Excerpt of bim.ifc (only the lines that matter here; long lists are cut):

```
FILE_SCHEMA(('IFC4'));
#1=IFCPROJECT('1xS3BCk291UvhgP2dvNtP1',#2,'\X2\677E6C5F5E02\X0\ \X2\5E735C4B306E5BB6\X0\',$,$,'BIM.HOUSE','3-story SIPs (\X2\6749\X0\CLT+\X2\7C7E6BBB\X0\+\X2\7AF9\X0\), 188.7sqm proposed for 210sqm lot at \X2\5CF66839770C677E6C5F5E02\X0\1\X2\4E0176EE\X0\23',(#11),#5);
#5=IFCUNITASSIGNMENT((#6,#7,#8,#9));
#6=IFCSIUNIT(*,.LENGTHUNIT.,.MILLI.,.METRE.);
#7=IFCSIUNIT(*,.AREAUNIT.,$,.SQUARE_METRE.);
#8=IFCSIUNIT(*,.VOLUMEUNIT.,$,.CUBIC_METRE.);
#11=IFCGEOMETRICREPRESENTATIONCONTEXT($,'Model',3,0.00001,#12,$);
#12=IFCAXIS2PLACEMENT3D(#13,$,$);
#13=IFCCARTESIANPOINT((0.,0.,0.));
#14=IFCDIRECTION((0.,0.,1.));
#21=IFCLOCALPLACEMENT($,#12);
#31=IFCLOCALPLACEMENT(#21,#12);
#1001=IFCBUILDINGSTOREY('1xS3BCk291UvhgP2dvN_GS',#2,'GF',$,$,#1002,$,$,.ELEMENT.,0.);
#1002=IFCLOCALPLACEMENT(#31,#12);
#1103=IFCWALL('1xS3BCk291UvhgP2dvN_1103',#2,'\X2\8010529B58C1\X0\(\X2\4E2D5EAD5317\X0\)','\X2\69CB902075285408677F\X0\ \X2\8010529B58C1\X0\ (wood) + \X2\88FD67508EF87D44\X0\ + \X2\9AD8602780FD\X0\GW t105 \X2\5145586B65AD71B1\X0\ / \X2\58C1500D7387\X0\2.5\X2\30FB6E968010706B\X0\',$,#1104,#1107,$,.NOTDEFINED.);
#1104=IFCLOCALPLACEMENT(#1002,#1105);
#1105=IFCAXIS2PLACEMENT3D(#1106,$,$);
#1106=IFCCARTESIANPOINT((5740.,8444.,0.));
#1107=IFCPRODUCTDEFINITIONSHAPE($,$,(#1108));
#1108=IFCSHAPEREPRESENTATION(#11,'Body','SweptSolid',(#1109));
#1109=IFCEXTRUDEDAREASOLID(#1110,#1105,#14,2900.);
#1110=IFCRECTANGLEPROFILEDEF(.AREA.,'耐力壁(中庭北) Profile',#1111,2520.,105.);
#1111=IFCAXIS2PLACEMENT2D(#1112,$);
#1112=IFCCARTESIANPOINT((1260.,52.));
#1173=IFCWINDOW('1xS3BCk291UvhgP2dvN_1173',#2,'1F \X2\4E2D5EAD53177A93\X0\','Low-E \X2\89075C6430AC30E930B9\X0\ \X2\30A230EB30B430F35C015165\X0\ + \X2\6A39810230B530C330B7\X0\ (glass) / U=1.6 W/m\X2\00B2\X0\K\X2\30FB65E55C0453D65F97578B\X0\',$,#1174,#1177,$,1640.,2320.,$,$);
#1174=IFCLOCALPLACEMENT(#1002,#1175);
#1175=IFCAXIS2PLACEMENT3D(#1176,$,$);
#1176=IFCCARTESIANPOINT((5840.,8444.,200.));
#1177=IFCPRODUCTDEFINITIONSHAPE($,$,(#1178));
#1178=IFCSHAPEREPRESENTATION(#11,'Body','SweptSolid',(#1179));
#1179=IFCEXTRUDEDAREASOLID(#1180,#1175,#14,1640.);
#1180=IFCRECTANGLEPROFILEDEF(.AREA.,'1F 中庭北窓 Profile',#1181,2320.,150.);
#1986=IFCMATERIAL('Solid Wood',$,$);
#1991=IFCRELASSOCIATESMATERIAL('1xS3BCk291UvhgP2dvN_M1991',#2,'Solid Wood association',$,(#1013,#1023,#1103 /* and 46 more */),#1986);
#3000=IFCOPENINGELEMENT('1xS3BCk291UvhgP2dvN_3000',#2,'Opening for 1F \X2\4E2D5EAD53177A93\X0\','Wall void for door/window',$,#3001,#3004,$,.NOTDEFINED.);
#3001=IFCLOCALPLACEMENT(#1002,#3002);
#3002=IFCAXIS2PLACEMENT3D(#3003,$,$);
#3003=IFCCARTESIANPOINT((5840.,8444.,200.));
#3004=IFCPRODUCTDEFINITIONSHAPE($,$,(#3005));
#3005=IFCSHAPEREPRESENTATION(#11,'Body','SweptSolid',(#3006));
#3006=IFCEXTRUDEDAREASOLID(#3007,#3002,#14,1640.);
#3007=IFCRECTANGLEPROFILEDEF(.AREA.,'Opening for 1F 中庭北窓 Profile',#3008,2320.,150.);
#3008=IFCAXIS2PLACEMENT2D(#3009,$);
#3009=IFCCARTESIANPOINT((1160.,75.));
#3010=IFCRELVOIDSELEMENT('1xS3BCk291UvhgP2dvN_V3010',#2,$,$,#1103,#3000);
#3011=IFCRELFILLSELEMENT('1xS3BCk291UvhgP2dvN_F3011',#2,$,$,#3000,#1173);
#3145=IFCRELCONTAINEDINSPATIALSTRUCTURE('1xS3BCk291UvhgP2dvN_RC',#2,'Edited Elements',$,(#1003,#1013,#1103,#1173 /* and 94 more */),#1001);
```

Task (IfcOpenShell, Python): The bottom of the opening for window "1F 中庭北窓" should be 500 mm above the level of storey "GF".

```python
import numpy as np
import ifcopenshell
import ifcopenshell.api.geometry
import ifcopenshell.geom
import ifcopenshell.util.element
import ifcopenshell.util.placement
import ifcopenshell.util.shape
import ifcopenshell.util.unit

model = ifcopenshell.open("bim.ifc")
unit_scale = ifcopenshell.util.unit.calculate_unit_scale(model)

window = model.by_guid("1xS3BCk291UvhgP2dvN_1173")
opening = window.FillsVoids[0].RelatingOpeningElement
storey = ifcopenshell.util.element.get_container(window, ifc_class="IfcBuildingStorey")
level = ifcopenshell.util.placement.get_local_placement(storey.ObjectPlacement)[2, 3]

# The opening's origin need not be at the sill, so measure its lowest point.
shape = ifcopenshell.geom.create_shape(ifcopenshell.geom.settings(), opening)
bottom = ifcopenshell.util.shape.get_shape_bottom_elevation(shape, shape.geometry) / unit_scale
dz = level + 0.5 / unit_scale - bottom

shift = np.array([0.0, 0.0, dz])
# The window is not placed relative to its opening, so move both.
for product in (opening, window):
    matrix = ifcopenshell.util.placement.get_local_placement(product.ObjectPlacement)
    matrix[:3, 3] += shift
    ifcopenshell.api.geometry.edit_object_placement(model, product=product, matrix=matrix, is_si=False)

print(f"moved by {dz * unit_scale:+.3f} m")

model.write("bim_v2.ifc")
```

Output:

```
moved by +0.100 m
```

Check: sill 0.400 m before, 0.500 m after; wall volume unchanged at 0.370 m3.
